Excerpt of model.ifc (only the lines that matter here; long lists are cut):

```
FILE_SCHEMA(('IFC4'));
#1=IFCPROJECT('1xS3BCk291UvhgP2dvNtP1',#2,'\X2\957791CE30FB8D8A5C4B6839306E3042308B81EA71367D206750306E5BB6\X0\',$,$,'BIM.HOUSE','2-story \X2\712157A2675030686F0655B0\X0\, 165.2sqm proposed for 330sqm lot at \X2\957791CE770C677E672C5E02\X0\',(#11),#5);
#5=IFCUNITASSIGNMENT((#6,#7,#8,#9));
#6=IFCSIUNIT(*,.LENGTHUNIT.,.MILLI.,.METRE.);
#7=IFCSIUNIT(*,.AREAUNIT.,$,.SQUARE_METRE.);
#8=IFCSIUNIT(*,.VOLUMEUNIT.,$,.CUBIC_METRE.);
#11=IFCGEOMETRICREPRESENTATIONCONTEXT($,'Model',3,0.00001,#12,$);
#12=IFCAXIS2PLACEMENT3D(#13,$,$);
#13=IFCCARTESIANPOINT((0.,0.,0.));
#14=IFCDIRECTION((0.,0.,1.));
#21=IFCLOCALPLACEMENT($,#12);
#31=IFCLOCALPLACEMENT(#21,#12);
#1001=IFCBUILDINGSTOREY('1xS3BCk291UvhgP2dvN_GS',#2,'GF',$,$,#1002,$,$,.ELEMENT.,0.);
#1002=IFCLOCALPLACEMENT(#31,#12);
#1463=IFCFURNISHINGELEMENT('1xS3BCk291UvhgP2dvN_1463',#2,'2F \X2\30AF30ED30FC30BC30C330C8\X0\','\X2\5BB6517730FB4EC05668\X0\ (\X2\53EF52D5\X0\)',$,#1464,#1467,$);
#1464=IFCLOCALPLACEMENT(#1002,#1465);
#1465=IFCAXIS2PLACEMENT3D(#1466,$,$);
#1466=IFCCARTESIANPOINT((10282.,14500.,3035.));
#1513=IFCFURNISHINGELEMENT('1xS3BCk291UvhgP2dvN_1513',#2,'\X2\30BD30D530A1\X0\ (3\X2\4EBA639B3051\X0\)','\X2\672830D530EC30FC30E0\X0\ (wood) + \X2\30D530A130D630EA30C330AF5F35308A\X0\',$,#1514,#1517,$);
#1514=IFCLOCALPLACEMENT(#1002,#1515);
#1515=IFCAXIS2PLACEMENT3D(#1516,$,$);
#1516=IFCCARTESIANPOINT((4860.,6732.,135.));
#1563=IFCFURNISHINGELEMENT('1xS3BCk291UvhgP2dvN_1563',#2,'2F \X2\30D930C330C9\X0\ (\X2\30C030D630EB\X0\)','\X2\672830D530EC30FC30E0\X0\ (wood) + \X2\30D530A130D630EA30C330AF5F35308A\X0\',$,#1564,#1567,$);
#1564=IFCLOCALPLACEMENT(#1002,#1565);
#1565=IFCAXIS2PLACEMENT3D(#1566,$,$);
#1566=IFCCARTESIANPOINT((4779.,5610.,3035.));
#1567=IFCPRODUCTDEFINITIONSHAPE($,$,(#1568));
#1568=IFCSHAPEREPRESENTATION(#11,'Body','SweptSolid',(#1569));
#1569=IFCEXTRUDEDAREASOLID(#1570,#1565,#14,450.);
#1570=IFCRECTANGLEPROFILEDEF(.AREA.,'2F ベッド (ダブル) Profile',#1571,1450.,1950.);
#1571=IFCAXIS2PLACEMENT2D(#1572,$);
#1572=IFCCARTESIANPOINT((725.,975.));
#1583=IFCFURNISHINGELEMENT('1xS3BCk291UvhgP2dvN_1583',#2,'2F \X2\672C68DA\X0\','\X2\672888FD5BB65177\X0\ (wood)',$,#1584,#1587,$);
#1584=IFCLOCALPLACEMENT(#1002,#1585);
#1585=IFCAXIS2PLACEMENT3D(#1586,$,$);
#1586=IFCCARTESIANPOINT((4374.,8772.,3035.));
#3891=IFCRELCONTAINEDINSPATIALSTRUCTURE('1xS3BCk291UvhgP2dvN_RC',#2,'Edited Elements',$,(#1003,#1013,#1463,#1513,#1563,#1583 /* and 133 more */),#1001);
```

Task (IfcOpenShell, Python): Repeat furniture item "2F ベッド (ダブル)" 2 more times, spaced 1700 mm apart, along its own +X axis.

```python
import ifcopenshell
import ifcopenshell.api.geometry
import ifcopenshell.api.root
import ifcopenshell.util.element
import ifcopenshell.util.placement
import ifcopenshell.util.unit

model = ifcopenshell.open("model.ifc")
unit_scale = ifcopenshell.util.unit.calculate_unit_scale(model)


def reuse_history(source, copy):
    """copy_class also copies each property set's owner history, people and application; keep the originals."""
    for rel in copy.IsDefinedBy:
        if rel.is_a("IfcRelDefinesByProperties") and (history := rel.RelatingPropertyDefinition.OwnerHistory):
            rel.RelatingPropertyDefinition.OwnerHistory = source.OwnerHistory
            ifcopenshell.util.element.remove_deep2(model, history)


source = model.by_guid("1xS3BCk291UvhgP2dvN_1563")
base = ifcopenshell.util.placement.get_local_placement(source.ObjectPlacement)
step = base[:3, 0] * 1.7 / unit_scale

for i in range(1, 3):
    copy = ifcopenshell.api.root.copy_class(model, product=source)
    copy.Representation = ifcopenshell.util.element.copy_deep(
        model, source.Representation, exclude=["IfcGeometricRepresentationContext", "IfcRepresentationMap"]
    )
    reuse_history(source, copy)
    matrix = base.copy()
    matrix[:3, 3] += i * step
    print("added at", matrix[:3, 3].round(3) + 0.0)
    ifcopenshell.api.geometry.edit_object_placement(model, product=copy, matrix=matrix, is_si=False)

model.write("model_rev.ifc")
```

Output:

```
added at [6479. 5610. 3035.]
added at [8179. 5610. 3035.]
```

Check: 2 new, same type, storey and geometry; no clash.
